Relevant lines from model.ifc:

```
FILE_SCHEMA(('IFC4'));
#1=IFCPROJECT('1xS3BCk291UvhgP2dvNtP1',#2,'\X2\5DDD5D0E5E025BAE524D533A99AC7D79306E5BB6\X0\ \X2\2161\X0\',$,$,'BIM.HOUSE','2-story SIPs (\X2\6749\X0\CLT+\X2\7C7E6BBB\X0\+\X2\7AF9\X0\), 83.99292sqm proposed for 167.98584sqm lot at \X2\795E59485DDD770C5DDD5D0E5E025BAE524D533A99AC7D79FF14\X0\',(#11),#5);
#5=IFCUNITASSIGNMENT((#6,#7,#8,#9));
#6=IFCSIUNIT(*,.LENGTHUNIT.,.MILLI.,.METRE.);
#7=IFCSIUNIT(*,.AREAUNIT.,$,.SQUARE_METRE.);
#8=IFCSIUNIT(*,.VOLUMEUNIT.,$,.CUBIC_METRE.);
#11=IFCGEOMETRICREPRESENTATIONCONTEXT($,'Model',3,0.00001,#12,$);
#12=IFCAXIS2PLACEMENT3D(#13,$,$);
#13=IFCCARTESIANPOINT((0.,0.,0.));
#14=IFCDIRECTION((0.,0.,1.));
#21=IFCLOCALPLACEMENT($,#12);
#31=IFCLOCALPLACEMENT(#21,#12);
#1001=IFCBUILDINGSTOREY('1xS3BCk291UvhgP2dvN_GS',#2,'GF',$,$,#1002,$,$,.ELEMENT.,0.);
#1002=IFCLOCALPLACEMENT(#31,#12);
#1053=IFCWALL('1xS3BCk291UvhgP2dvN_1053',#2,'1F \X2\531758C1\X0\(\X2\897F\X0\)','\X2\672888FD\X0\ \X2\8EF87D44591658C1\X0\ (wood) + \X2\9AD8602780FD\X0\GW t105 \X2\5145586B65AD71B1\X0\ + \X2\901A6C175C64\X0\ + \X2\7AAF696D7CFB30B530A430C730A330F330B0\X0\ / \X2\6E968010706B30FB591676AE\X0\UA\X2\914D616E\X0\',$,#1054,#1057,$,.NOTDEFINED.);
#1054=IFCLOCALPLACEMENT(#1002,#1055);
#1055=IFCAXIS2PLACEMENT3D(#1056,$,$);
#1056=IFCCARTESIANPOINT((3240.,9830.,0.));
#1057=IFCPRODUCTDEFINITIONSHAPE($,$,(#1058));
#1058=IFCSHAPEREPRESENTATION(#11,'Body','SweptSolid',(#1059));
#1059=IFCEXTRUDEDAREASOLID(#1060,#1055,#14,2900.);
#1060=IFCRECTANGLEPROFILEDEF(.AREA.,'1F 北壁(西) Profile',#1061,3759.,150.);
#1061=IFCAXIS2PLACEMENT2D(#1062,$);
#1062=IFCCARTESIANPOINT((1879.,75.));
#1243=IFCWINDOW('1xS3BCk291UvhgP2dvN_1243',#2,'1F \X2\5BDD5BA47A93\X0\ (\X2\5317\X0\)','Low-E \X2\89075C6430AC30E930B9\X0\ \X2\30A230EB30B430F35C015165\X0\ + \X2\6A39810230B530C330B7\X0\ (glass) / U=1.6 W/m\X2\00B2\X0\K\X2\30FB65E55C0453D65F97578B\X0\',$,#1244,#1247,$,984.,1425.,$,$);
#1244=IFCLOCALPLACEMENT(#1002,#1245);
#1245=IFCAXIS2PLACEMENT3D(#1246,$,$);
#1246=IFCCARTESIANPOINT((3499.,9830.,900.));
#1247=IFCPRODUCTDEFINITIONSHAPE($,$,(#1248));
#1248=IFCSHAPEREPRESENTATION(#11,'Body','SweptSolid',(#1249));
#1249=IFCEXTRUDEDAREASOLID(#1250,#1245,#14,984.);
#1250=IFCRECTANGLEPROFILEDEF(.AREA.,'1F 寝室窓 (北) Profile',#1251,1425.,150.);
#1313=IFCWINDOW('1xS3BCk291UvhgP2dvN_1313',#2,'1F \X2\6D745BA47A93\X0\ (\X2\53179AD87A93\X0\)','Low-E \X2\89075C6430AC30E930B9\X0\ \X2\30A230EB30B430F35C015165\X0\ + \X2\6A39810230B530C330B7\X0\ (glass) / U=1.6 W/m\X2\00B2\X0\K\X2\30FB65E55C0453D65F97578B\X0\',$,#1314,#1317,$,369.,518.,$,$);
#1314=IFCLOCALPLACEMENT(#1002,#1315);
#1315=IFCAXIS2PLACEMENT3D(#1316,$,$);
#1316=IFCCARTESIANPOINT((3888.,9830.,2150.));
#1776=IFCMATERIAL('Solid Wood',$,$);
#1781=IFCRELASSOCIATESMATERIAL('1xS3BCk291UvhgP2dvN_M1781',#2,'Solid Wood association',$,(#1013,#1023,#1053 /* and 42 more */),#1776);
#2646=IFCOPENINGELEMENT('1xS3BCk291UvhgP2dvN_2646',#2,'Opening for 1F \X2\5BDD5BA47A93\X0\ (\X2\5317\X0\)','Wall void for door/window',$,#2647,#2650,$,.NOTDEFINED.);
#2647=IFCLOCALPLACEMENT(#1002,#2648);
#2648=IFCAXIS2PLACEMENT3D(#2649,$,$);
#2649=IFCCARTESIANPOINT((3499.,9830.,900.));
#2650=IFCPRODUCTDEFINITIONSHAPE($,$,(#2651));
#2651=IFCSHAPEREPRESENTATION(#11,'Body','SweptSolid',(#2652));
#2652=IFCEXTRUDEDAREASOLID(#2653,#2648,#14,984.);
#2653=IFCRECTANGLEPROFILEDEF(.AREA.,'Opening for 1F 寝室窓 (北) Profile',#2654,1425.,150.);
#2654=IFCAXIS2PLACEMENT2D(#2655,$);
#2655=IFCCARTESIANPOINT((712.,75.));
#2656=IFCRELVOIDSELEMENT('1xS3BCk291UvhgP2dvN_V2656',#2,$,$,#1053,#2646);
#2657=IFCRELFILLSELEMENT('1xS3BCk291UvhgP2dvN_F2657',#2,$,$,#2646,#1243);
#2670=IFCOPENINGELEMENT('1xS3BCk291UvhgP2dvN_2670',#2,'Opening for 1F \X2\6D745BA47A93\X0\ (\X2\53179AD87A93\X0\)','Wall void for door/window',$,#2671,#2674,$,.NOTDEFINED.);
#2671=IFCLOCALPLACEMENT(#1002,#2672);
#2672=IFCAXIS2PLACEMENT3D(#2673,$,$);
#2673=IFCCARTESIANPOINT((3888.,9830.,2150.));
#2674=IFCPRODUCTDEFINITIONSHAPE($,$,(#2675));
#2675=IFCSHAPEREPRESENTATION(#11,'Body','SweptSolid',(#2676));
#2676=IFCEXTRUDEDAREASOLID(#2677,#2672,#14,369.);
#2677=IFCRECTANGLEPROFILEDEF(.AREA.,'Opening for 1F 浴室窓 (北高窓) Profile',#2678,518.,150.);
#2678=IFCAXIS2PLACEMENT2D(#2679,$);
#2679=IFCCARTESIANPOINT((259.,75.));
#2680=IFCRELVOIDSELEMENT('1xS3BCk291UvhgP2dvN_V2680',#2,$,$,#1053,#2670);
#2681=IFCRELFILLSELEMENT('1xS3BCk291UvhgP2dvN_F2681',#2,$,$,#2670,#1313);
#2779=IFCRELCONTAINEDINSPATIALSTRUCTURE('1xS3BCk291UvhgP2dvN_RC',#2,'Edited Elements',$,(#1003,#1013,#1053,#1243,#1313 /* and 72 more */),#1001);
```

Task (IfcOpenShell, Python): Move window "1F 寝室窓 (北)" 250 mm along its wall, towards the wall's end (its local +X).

```python
import ifcopenshell
import ifcopenshell.api.geometry
import ifcopenshell.util.placement

model = ifcopenshell.open("model.ifc")

window = model.by_id(1243)
opening = window.FillsVoids[0].RelatingOpeningElement
wall = opening.VoidsElements[0].RelatingBuildingElement

wall_matrix = ifcopenshell.util.placement.get_local_placement(wall.ObjectPlacement)
shift = wall_matrix[:3, 0] * 250.0
before = ifcopenshell.util.placement.get_local_placement(window.ObjectPlacement)[:3, 3].copy()

# The window is not placed relative to its opening, so move both.
for product in (opening, window):
    matrix = ifcopenshell.util.placement.get_local_placement(product.ObjectPlacement)
    matrix[:3, 3] += shift
    ifcopenshell.api.geometry.edit_object_placement(model, product=product, matrix=matrix, is_si=False)

after = ifcopenshell.util.placement.get_local_placement(window.ObjectPlacement)[:3, 3]
print("window moved by", (after - before).round(3) + 0.0)

model.write("model-out.ifc")
```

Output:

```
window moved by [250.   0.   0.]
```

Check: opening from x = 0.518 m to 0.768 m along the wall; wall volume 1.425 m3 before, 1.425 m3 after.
